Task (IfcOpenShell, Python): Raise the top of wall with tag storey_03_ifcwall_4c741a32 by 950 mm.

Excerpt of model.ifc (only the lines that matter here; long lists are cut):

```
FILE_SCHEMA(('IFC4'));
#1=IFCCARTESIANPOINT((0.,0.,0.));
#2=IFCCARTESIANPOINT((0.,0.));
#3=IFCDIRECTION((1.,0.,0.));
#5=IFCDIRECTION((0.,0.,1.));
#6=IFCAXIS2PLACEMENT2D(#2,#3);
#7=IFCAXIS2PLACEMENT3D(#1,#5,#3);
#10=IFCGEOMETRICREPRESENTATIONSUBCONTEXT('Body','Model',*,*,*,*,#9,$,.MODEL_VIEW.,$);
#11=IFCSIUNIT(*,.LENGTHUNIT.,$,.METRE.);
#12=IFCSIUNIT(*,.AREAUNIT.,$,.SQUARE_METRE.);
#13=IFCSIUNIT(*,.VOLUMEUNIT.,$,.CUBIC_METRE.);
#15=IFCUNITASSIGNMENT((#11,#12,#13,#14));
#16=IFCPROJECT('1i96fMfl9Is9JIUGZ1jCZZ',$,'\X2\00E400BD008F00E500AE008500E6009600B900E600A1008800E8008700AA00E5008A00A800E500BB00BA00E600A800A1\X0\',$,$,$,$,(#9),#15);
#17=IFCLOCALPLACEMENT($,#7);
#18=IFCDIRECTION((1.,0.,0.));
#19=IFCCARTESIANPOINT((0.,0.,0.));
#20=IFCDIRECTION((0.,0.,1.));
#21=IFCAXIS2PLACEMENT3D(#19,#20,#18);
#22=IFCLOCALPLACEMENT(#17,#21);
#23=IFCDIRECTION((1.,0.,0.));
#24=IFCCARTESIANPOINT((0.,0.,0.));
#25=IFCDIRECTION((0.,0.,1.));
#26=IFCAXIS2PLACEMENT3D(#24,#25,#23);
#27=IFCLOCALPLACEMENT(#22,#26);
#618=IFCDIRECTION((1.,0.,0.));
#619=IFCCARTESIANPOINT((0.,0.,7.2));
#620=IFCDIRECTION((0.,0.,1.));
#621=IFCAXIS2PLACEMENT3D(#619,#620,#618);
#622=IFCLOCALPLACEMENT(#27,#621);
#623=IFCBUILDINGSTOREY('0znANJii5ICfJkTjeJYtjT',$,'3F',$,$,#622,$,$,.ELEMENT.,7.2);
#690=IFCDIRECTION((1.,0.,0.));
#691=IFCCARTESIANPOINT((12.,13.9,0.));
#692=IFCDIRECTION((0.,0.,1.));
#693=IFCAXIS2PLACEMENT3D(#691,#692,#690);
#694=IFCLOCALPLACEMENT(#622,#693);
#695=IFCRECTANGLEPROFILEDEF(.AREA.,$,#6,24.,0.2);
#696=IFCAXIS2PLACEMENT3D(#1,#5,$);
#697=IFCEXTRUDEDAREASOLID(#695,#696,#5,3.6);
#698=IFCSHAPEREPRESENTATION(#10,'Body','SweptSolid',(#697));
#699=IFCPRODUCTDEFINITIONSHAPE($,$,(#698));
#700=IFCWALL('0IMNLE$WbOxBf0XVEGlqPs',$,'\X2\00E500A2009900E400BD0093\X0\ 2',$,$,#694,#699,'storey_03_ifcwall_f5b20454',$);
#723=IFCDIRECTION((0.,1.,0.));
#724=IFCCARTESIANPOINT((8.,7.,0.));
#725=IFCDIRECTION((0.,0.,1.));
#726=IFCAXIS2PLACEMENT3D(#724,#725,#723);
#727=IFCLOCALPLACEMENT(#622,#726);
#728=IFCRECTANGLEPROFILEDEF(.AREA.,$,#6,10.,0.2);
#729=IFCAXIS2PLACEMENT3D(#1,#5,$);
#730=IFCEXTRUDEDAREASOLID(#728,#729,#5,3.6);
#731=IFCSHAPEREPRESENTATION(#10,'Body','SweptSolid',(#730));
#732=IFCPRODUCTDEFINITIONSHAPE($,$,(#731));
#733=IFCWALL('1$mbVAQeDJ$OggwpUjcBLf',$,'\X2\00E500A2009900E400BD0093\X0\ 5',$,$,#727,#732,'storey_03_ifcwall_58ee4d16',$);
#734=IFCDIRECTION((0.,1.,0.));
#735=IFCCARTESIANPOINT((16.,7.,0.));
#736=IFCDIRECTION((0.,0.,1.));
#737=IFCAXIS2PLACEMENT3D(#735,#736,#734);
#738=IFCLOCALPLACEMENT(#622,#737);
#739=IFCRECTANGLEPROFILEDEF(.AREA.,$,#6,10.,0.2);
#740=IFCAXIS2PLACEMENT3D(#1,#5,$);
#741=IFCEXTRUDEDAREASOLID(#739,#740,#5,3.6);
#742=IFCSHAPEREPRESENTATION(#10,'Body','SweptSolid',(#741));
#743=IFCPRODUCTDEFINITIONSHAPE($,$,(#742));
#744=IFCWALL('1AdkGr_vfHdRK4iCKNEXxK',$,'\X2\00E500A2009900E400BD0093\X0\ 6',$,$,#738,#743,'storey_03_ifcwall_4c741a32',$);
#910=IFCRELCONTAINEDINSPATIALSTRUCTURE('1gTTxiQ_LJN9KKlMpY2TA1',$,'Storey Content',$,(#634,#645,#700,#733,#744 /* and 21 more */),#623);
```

```python
import ifcopenshell
import ifcopenshell.geom
import ifcopenshell.util.representation
import ifcopenshell.util.shape

model = ifcopenshell.open("model.ifc")
settings = ifcopenshell.geom.settings()


def volume(element):
    """Net volume in cubic metres, openings subtracted."""
    shape = ifcopenshell.geom.create_shape(settings, element)
    return ifcopenshell.util.shape.get_volume(shape.geometry)


wall = model.by_guid("1AdkGr_vfHdRK4iCKNEXxK")
before = volume(wall)

body = ifcopenshell.util.representation.get_representation(wall, "Model", "Body")
solid = body.Items[0]
old_height = solid.Depth
solid.Depth += 0.95
after = volume(wall)

print(f"height {old_height:g} -> {solid.Depth:g}, volume {before:.3f} -> {after:.3f} m3")

model.write("model-out.ifc")
```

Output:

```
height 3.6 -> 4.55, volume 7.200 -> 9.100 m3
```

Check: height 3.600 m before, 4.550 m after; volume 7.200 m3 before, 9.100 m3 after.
